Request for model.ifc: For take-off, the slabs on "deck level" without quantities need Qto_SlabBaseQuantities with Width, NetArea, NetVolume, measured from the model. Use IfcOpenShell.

First a look at what the model holds.

```python
import ifcopenshell
import ifcopenshell.util.element
import ifcopenshell.util.unit

model = ifcopenshell.open("model.ifc")
print(model.schema)
for unit_type in ("LENGTHUNIT", "AREAUNIT", "VOLUMEUNIT"):
    print(unit_type, ifcopenshell.util.unit.calculate_unit_scale(model, unit_type))
storey = next(s for s in model.by_type("IfcBuildingStorey") if s.Name == "deck level")
slabs = [e for e in ifcopenshell.util.element.get_decomposition(storey) if e.is_a("IfcSlab")]
for e in sorted(slabs, key=lambda e: e.id()):
    print(e.id(), e.is_a(), e.Name, list(ifcopenshell.util.element.get_psets(e, qtos_only=True)), sep=" | ")
```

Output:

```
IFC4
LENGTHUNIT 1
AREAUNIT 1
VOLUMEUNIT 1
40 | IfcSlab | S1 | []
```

```python
import ifcopenshell
import ifcopenshell.api.pset
import ifcopenshell.geom
import ifcopenshell.util.element
import ifcopenshell.util.shape
import ifcopenshell.util.unit

model = ifcopenshell.open("model.ifc")
unit_scale = ifcopenshell.util.unit.calculate_unit_scale(model)
area_scale = ifcopenshell.util.unit.calculate_unit_scale(model, "AREAUNIT")
volume_scale = ifcopenshell.util.unit.calculate_unit_scale(model, "VOLUMEUNIT")
settings = ifcopenshell.geom.settings()

storey = next(s for s in model.by_type("IfcBuildingStorey") if s.Name == "deck level")
slabs = [e for e in ifcopenshell.util.element.get_decomposition(storey) if e.is_a("IfcSlab")]

for e in sorted(slabs, key=lambda e: e.id()):
    if ifcopenshell.util.element.get_psets(e, qtos_only=True, should_inherit=False):
        continue
    # Geometry comes back in metres, in the element's own axes.
    shape = ifcopenshell.geom.create_shape(settings, e)
    values = {
        "Width": ifcopenshell.util.shape.get_z(shape.geometry) / unit_scale,
        "NetArea": ifcopenshell.util.shape.get_footprint_area(shape.geometry) / area_scale,
        "NetVolume": ifcopenshell.util.shape.get_volume(shape.geometry) / volume_scale,
    }
    qto = ifcopenshell.api.pset.add_qto(model, product=e, name="Qto_SlabBaseQuantities")
    ifcopenshell.api.pset.edit_qto(model, qto=qto, properties=values)
    print(e.id(), {k: round(v, 3) for k, v in values.items()})

model.write("model_edited.ifc")
```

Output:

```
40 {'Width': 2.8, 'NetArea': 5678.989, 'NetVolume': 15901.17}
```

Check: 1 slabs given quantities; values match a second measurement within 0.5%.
